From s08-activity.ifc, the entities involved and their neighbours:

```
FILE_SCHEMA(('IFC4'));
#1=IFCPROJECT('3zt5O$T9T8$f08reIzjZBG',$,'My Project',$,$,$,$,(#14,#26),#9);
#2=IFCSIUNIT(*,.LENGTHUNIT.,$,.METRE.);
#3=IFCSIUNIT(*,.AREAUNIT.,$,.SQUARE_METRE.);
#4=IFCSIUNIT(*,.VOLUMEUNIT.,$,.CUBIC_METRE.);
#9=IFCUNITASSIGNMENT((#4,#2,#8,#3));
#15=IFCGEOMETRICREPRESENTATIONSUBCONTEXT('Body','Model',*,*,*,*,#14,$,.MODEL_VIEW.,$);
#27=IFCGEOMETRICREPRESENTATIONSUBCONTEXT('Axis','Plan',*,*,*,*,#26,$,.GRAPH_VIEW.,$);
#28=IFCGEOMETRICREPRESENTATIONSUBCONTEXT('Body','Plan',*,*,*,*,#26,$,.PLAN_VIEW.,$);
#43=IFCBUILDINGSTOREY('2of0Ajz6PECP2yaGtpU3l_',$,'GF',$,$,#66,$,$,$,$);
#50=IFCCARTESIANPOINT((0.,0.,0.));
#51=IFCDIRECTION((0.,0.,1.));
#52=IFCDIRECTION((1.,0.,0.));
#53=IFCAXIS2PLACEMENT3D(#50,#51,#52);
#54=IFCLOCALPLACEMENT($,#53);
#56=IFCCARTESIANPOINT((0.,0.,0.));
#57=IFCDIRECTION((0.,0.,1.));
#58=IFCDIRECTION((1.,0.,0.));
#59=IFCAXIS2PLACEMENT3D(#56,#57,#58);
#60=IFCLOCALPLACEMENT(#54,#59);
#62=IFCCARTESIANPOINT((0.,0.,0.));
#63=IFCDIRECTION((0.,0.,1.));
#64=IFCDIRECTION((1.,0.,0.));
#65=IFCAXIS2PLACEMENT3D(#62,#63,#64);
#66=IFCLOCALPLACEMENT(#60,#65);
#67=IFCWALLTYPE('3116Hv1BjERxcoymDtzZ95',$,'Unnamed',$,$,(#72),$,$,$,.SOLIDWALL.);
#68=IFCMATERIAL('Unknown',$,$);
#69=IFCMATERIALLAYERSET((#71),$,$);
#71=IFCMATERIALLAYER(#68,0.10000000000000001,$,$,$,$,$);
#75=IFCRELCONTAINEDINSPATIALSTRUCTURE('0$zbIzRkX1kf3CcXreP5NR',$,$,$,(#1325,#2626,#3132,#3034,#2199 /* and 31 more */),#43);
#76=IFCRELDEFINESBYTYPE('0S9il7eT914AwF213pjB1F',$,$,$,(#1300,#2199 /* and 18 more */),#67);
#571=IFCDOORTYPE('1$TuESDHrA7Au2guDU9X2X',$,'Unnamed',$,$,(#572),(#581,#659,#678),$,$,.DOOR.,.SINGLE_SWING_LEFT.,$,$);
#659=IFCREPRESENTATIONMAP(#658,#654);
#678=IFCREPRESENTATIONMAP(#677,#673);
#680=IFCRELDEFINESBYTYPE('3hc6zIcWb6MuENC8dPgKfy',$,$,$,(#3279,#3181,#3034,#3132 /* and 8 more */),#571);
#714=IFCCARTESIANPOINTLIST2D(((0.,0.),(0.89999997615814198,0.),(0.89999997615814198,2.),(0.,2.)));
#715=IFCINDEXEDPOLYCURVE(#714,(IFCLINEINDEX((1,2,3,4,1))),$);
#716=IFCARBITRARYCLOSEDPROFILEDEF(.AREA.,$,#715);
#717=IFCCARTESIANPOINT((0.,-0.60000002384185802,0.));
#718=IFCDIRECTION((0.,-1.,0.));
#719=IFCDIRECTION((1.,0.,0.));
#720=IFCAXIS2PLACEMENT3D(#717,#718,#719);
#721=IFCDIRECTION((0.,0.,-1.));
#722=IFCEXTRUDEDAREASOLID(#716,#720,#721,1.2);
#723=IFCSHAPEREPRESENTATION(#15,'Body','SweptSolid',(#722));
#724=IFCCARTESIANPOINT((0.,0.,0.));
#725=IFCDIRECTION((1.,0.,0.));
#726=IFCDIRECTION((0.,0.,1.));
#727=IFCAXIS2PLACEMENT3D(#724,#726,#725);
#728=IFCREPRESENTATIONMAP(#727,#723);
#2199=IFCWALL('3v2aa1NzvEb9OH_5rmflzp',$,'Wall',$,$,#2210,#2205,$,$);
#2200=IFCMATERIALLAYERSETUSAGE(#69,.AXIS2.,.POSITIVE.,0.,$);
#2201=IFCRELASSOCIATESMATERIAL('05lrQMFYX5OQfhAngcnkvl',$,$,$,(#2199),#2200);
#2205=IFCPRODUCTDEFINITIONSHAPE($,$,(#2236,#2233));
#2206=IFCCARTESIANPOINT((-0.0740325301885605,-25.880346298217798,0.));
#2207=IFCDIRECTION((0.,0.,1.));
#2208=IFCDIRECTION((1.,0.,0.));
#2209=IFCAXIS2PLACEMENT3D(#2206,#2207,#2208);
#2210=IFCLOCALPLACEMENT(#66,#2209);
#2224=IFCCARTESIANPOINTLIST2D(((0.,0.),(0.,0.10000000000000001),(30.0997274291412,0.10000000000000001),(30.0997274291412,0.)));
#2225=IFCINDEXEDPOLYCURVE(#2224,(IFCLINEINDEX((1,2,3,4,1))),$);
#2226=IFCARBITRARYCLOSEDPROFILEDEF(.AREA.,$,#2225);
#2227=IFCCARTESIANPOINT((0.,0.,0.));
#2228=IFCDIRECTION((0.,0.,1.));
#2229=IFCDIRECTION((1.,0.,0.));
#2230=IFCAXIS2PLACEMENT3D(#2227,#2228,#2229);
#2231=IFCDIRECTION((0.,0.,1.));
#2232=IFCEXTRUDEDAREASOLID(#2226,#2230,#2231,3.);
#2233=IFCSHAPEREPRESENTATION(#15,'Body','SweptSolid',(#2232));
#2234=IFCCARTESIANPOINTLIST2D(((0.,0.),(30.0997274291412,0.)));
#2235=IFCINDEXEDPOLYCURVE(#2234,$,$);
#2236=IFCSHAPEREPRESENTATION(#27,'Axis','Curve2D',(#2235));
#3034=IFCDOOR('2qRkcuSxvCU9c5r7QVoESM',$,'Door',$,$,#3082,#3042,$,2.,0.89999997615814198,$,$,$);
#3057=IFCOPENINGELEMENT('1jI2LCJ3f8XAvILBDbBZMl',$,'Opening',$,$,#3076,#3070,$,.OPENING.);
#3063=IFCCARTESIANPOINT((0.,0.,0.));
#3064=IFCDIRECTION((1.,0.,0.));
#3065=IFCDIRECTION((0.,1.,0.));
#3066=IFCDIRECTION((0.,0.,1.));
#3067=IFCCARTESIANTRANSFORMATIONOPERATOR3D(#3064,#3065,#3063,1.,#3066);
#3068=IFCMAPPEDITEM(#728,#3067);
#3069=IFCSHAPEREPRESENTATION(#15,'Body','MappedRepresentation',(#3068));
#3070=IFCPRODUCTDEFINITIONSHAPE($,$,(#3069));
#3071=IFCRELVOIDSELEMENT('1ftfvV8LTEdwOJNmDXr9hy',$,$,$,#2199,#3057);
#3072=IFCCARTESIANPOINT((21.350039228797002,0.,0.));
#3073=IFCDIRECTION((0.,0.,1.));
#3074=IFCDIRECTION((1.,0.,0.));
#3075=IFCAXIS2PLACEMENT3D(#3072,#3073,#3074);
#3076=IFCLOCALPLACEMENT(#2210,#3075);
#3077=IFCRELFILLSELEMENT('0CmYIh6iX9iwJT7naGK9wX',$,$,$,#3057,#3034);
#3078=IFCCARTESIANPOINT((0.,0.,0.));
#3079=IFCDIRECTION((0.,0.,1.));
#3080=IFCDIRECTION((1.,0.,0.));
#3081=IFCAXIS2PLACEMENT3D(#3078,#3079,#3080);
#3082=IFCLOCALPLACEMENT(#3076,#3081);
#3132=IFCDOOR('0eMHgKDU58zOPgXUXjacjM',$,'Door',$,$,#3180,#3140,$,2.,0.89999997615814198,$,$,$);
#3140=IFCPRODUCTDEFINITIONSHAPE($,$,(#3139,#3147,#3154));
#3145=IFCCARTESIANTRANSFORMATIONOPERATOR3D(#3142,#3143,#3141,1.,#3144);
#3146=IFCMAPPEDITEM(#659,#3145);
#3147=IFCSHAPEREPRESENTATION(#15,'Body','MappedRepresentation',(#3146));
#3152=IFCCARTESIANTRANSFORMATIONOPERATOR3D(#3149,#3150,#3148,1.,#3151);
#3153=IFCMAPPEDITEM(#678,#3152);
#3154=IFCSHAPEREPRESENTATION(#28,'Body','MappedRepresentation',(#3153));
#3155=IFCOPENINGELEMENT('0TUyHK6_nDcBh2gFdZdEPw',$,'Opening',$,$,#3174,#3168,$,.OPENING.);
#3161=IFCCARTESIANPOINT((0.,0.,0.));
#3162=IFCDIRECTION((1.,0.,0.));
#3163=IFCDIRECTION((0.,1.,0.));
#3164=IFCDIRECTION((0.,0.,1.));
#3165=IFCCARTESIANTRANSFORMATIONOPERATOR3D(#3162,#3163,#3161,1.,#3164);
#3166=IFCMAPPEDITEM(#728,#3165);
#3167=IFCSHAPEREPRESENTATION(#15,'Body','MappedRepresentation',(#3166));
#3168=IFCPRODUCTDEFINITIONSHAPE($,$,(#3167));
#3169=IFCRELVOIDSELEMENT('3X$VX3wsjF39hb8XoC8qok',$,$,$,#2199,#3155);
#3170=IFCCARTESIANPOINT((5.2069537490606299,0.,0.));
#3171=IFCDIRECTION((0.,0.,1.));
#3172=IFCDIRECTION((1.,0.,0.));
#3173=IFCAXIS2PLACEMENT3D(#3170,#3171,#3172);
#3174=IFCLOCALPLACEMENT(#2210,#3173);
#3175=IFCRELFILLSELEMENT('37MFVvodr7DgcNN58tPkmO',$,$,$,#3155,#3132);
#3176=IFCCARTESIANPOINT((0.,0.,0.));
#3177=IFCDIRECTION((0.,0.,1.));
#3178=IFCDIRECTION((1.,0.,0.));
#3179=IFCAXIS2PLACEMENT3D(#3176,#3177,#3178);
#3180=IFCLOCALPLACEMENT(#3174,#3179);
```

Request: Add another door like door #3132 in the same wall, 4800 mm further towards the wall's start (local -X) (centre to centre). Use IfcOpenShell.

```python
import ifcopenshell
import ifcopenshell.api.feature
import ifcopenshell.api.geometry
import ifcopenshell.api.root
import ifcopenshell.geom
import ifcopenshell.util.element
import ifcopenshell.util.placement
import ifcopenshell.util.shape

model = ifcopenshell.open("s08-activity.ifc")
settings = ifcopenshell.geom.settings()


def volume(element):
    """Net volume in cubic metres, openings subtracted."""
    shape = ifcopenshell.geom.create_shape(settings, element)
    return ifcopenshell.util.shape.get_volume(shape.geometry)


door = model.by_id(3132)
opening = door.FillsVoids[0].RelatingOpeningElement
wall = opening.VoidsElements[0].RelatingBuildingElement
before = volume(wall)
shift = ifcopenshell.util.placement.get_local_placement(wall.ObjectPlacement)[:3, 0] * -4.8

# copy_class copies the void relationship, type, container and properties, but no geometry.
new_opening = ifcopenshell.api.root.copy_class(model, product=opening)
new_opening.Representation = ifcopenshell.util.element.copy_deep(
    model, opening.Representation, exclude=["IfcGeometricRepresentationContext", "IfcRepresentationMap"]
)
new_door = ifcopenshell.api.root.copy_class(model, product=door)
new_door.Representation = ifcopenshell.util.element.copy_deep(
    model, door.Representation, exclude=["IfcGeometricRepresentationContext", "IfcRepresentationMap"]
)
ifcopenshell.api.feature.add_filling(model, opening=new_opening, element=new_door)

for old, new in ((opening, new_opening), (door, new_door)):
    matrix = ifcopenshell.util.placement.get_local_placement(old.ObjectPlacement)
    matrix[:3, 3] += shift
    ifcopenshell.api.geometry.edit_object_placement(model, product=new, matrix=matrix, is_si=False)

after = volume(wall)

print(f"wall volume {before:.3f} -> {after:.3f} m3")

model.write("s08-activity_edited.ifc")
```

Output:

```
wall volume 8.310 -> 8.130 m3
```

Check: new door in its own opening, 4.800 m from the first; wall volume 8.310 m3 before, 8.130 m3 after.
